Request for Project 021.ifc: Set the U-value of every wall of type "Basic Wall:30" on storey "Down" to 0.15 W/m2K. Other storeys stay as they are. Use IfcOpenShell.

First a look at what the model holds.

```python
import ifcopenshell
import ifcopenshell.util.element

model = ifcopenshell.open("Project 021.ifc")
print(model.schema)
storey = next(s for s in model.by_type("IfcBuildingStorey") if s.Name == "Down")
walls = [e for e in ifcopenshell.util.element.get_decomposition(storey) if e.is_a("IfcWall")]
seen = {}
for e in walls:
    element_type = ifcopenshell.util.element.get_type(e)
    key = (element_type.Name if element_type != e and element_type else None, ifcopenshell.util.element.get_pset(e, "Pset_WallCommon", "ThermalTransmittance"))
    seen[key] = seen.get(key, 0) + 1
for (name, value), count in sorted(seen.items(), key=str):
    print(count, "x", name, "|", value)
```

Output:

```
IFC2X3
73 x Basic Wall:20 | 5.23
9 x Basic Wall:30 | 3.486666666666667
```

```python
import ifcopenshell
import ifcopenshell.api.pset
import ifcopenshell.util.element

model = ifcopenshell.open("Project 021.ifc")

storey = next(s for s in model.by_type("IfcBuildingStorey") if s.Name == "Down")
walls = [e for e in ifcopenshell.util.element.get_decomposition(storey) if e.is_a("IfcWall")]

count = 0
for e in walls:
    element_type = ifcopenshell.util.element.get_type(e)
    if element_type in (None, e) or element_type.Name != "Basic Wall:30":
        continue
    # add_pset returns the element's existing set when there is one.
    pset = ifcopenshell.api.pset.add_pset(model, product=e, name="Pset_WallCommon")
    ifcopenshell.api.pset.edit_pset(model, pset=pset, properties={"ThermalTransmittance": 0.15})
    count += 1

print(count, "walls updated")

model.write("Project 021_edited.ifc")
```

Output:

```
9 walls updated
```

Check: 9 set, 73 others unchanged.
